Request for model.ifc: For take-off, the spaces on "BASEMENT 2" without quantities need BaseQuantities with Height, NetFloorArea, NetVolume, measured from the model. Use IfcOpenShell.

First a look at what the model holds.

```python
import ifcopenshell
import ifcopenshell.util.element
import ifcopenshell.util.unit

model = ifcopenshell.open("model.ifc")
print(model.schema)
for unit_type in ("LENGTHUNIT", "AREAUNIT", "VOLUMEUNIT"):
    print(unit_type, ifcopenshell.util.unit.calculate_unit_scale(model, unit_type))
storey = next(s for s in model.by_type("IfcBuildingStorey") if s.Name == "BASEMENT 2")
spaces = [e for e in ifcopenshell.util.element.get_decomposition(storey) if e.is_a("IfcSpace")]
for e in sorted(spaces, key=lambda e: e.id()):
    print(e.id(), e.is_a(), e.Name, list(ifcopenshell.util.element.get_psets(e, qtos_only=True)), sep=" | ")
```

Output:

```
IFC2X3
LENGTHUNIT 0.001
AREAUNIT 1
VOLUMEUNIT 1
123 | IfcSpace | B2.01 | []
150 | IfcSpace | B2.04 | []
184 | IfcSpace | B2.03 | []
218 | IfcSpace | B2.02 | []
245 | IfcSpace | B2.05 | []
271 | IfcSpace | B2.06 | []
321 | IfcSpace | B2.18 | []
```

```python
import ifcopenshell
import ifcopenshell.api.pset
import ifcopenshell.geom
import ifcopenshell.util.element
import ifcopenshell.util.shape
import ifcopenshell.util.unit

model = ifcopenshell.open("model.ifc")
unit_scale = ifcopenshell.util.unit.calculate_unit_scale(model)
area_scale = ifcopenshell.util.unit.calculate_unit_scale(model, "AREAUNIT")
volume_scale = ifcopenshell.util.unit.calculate_unit_scale(model, "VOLUMEUNIT")
settings = ifcopenshell.geom.settings()

storey = next(s for s in model.by_type("IfcBuildingStorey") if s.Name == "BASEMENT 2")
spaces = [e for e in ifcopenshell.util.element.get_decomposition(storey) if e.is_a("IfcSpace")]

for e in sorted(spaces, key=lambda e: e.id()):
    if ifcopenshell.util.element.get_psets(e, qtos_only=True, should_inherit=False):
        continue
    # Geometry comes back in metres, in the element's own axes.
    shape = ifcopenshell.geom.create_shape(settings, e)
    values = {
        "Height": ifcopenshell.util.shape.get_z(shape.geometry) / unit_scale,
        "NetFloorArea": ifcopenshell.util.shape.get_footprint_area(shape.geometry) / area_scale,
        "NetVolume": ifcopenshell.util.shape.get_volume(shape.geometry) / volume_scale,
    }
    qto = ifcopenshell.api.pset.add_qto(model, product=e, name="BaseQuantities")
    ifcopenshell.api.pset.edit_qto(model, qto=qto, properties=values)
    print(e.id(), {k: round(v, 3) for k, v in values.items()})

model.write("model-out.ifc")
```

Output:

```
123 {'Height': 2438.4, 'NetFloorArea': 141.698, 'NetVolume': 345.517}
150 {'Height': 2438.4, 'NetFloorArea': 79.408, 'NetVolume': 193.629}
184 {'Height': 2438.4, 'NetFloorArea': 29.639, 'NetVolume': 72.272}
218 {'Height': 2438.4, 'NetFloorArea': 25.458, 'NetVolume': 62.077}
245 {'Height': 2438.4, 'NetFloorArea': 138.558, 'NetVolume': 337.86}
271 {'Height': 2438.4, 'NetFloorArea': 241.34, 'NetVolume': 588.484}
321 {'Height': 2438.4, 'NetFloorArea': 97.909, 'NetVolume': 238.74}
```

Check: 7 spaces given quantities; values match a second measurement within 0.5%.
